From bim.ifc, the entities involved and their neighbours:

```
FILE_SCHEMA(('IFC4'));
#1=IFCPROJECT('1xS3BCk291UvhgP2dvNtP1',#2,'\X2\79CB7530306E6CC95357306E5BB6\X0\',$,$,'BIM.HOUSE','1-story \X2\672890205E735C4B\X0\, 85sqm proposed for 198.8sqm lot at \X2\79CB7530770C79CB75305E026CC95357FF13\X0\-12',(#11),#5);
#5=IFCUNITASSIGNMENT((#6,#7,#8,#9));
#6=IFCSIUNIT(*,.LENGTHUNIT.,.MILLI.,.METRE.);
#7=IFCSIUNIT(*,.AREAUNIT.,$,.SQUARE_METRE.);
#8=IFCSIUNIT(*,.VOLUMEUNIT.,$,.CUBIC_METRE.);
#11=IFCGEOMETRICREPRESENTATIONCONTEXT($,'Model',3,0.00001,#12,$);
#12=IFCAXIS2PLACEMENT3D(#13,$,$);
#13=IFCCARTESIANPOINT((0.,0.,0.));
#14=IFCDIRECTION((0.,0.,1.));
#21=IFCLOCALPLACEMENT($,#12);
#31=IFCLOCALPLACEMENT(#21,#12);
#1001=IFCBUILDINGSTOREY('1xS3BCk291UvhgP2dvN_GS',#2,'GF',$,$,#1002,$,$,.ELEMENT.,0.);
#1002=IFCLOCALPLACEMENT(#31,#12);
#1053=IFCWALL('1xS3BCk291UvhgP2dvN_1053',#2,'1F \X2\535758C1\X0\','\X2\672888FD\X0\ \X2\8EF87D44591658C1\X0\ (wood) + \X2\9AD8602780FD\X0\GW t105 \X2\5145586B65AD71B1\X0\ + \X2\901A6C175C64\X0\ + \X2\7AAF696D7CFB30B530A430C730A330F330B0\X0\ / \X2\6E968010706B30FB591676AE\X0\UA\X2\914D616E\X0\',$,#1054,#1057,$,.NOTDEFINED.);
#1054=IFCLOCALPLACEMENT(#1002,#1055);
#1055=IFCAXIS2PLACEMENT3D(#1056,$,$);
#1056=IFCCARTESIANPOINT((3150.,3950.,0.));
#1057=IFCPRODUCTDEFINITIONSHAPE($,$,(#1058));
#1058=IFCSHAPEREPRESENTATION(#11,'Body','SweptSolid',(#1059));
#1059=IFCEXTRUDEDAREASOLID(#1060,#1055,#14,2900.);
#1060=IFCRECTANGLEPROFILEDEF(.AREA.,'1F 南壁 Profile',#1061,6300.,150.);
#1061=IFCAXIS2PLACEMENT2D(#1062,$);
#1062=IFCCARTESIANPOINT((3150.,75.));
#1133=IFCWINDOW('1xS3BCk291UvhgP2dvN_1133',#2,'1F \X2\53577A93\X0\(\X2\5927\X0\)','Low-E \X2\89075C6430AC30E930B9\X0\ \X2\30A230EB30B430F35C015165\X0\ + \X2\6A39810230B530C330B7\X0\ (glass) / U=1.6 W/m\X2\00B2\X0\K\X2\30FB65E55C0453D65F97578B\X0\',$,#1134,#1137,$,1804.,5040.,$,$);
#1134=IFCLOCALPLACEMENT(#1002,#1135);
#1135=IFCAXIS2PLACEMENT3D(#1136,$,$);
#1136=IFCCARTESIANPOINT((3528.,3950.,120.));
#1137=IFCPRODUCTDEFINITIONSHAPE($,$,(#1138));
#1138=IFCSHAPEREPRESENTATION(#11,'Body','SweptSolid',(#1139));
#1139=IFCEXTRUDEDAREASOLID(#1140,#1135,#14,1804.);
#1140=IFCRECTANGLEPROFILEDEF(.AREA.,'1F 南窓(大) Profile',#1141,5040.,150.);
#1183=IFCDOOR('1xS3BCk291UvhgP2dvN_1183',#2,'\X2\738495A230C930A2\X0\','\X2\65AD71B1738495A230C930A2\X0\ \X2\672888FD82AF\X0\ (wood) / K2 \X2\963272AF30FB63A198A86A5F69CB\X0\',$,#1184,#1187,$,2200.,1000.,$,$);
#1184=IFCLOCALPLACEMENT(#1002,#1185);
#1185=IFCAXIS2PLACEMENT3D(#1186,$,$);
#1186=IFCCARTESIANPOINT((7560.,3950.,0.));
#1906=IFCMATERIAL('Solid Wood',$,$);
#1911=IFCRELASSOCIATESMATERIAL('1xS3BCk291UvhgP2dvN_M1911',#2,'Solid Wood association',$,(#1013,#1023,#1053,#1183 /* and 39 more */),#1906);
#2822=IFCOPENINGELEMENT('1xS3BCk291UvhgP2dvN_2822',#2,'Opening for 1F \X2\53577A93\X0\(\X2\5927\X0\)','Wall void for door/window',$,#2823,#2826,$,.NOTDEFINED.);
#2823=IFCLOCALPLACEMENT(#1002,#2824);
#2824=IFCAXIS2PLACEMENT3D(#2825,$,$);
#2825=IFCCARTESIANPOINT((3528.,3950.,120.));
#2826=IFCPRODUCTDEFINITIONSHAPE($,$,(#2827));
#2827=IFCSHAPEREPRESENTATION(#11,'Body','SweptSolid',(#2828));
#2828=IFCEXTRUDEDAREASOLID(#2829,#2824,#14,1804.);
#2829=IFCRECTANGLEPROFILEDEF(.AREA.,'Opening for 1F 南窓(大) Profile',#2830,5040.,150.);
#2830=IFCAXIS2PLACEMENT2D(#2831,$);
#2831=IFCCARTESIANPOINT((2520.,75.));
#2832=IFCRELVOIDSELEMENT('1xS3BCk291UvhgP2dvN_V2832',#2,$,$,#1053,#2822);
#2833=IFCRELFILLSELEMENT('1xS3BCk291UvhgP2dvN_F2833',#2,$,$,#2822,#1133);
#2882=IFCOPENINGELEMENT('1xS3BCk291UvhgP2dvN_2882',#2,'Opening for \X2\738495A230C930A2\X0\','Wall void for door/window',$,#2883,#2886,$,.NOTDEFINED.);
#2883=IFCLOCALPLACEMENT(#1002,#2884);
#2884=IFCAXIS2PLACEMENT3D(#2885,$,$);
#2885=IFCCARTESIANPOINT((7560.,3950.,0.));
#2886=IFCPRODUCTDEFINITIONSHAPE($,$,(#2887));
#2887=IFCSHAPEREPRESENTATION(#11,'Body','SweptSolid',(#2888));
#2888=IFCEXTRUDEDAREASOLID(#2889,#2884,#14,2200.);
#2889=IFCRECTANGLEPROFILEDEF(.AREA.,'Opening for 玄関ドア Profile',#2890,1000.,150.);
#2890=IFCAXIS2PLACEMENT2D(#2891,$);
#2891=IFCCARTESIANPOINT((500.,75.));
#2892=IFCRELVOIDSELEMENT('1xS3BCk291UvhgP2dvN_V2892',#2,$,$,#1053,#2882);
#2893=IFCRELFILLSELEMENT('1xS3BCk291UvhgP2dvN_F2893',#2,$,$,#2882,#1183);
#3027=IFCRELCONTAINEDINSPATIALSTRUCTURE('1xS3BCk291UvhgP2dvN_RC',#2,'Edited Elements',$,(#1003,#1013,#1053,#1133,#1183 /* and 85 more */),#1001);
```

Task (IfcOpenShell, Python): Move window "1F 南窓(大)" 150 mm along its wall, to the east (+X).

```python
import ifcopenshell
import ifcopenshell.api.geometry
import ifcopenshell.util.placement
import ifcopenshell.util.unit

model = ifcopenshell.open("bim.ifc")
unit_scale = ifcopenshell.util.unit.calculate_unit_scale(model)

window = model.by_guid("1xS3BCk291UvhgP2dvN_1133")
opening = window.FillsVoids[0].RelatingOpeningElement
wall = opening.VoidsElements[0].RelatingBuildingElement

wall_matrix = ifcopenshell.util.placement.get_local_placement(wall.ObjectPlacement)
shift = wall_matrix[:3, 0] * 0.15 / unit_scale
before = ifcopenshell.util.placement.get_local_placement(window.ObjectPlacement)[:3, 3].copy()

# The window is not placed relative to its opening, so move both.
for product in (opening, window):
    matrix = ifcopenshell.util.placement.get_local_placement(product.ObjectPlacement)
    matrix[:3, 3] += shift
    ifcopenshell.api.geometry.edit_object_placement(model, product=product, matrix=matrix, is_si=False)

after = ifcopenshell.util.placement.get_local_placement(window.ObjectPlacement)[:3, 3]
print("window moved by", (after - before).round(3) + 0.0)

model.write("bim_updated.ifc")
```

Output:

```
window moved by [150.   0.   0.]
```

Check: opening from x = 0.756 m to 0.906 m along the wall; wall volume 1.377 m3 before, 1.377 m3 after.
